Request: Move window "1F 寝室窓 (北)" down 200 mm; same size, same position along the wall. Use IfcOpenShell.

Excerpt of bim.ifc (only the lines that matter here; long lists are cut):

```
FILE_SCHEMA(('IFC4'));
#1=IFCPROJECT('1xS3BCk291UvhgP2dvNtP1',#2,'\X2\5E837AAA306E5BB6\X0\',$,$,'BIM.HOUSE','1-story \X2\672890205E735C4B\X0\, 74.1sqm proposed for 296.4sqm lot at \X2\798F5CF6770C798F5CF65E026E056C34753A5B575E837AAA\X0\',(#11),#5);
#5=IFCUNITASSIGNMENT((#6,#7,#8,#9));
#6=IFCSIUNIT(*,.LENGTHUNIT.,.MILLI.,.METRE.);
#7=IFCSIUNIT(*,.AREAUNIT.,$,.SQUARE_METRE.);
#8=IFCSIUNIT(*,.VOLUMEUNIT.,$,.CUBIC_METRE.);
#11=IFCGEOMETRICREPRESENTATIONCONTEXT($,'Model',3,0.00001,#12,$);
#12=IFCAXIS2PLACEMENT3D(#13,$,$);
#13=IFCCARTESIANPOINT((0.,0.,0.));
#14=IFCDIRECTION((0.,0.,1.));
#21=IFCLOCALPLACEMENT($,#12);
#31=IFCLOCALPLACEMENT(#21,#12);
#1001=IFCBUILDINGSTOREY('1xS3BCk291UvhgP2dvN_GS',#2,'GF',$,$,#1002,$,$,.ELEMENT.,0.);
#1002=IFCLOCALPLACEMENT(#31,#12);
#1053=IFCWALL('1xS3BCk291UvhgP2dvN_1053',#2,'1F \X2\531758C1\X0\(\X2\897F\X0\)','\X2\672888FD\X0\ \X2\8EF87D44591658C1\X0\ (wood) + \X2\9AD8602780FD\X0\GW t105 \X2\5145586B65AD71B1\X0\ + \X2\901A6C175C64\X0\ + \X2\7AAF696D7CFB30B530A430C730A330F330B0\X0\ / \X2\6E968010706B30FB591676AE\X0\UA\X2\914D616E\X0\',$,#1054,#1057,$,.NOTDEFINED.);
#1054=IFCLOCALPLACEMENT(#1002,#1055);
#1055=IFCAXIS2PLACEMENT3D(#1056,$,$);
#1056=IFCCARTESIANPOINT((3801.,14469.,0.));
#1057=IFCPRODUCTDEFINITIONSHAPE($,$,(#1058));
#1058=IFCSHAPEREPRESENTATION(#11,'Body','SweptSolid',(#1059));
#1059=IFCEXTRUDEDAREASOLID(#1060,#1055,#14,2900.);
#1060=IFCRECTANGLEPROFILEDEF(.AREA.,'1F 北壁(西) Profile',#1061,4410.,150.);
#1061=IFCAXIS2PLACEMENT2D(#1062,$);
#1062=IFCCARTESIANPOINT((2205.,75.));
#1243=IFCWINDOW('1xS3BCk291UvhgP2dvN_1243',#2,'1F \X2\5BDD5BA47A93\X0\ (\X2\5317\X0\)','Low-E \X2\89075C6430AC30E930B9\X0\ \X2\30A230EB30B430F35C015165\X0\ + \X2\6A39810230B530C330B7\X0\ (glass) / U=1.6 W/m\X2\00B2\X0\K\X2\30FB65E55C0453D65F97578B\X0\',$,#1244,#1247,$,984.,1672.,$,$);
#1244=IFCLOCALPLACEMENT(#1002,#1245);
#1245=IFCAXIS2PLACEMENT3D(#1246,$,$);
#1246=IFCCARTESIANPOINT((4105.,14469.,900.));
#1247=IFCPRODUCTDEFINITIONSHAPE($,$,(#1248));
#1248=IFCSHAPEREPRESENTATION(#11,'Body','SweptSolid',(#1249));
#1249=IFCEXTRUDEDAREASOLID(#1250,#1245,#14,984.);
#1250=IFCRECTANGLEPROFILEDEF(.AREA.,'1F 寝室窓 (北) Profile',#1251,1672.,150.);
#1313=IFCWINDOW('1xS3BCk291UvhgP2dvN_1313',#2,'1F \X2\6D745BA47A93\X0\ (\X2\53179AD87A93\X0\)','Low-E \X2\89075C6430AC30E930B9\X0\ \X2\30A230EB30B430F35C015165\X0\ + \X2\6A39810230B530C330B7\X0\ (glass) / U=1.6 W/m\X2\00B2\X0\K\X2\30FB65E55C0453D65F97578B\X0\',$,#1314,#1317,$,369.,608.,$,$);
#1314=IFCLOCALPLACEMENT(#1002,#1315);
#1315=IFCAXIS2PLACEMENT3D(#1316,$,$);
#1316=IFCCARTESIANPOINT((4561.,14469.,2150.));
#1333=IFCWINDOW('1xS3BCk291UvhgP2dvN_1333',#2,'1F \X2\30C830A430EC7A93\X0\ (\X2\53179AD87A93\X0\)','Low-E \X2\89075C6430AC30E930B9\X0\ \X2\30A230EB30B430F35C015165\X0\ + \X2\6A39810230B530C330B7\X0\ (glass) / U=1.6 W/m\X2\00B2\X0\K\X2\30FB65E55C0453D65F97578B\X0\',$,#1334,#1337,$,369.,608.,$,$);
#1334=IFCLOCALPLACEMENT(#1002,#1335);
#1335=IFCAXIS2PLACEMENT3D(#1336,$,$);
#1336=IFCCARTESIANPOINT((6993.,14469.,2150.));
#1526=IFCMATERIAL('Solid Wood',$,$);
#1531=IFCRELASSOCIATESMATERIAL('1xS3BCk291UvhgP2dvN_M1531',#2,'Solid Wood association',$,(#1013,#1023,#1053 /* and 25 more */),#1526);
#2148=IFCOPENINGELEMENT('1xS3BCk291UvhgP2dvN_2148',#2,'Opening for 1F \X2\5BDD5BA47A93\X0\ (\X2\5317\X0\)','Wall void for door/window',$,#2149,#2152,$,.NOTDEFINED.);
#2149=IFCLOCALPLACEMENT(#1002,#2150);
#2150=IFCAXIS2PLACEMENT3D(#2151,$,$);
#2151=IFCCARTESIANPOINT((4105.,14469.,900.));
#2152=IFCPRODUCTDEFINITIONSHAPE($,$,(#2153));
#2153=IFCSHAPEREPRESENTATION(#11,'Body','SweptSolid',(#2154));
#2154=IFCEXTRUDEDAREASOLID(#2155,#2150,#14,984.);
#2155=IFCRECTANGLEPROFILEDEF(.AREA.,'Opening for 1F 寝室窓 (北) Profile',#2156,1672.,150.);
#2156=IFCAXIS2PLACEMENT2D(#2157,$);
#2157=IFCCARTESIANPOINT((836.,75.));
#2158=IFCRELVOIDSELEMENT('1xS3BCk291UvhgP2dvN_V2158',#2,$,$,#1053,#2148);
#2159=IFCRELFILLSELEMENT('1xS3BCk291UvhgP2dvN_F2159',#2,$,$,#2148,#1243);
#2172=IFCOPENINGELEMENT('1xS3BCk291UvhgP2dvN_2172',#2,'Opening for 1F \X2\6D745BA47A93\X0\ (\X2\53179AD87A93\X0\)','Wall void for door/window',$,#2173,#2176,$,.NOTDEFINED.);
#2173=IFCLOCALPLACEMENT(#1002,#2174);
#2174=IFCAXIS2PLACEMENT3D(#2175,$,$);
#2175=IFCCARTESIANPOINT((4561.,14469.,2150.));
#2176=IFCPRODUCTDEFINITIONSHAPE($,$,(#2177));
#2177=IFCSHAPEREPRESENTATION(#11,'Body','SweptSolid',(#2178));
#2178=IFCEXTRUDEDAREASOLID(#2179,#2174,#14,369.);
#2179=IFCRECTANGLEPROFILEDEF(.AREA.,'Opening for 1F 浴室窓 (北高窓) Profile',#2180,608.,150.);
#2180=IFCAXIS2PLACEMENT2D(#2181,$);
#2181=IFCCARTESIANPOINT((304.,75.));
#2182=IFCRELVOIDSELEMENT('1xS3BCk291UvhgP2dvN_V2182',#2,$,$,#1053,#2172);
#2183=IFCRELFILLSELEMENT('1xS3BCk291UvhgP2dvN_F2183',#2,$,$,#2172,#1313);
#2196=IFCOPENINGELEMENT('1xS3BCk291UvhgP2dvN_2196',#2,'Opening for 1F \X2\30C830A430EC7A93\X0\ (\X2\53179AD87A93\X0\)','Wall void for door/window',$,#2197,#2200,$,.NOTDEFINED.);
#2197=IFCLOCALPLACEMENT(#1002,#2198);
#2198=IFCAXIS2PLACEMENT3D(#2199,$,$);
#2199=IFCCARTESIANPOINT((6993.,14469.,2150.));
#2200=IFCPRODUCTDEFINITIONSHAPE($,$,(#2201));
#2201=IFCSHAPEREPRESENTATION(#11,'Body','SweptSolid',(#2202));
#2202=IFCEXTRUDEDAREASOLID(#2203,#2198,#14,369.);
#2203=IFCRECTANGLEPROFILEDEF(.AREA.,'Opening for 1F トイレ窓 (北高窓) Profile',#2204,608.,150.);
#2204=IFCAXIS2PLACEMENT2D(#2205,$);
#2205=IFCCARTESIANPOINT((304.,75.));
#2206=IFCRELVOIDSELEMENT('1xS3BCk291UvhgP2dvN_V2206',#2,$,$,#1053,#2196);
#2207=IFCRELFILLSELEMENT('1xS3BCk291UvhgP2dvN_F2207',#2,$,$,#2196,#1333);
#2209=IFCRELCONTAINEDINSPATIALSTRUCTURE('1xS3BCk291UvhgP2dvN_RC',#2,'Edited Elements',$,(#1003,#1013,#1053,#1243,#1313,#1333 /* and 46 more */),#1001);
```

```python
import numpy as np
import ifcopenshell
import ifcopenshell.api.geometry
import ifcopenshell.util.placement
import ifcopenshell.util.unit

model = ifcopenshell.open("bim.ifc")
unit_scale = ifcopenshell.util.unit.calculate_unit_scale(model)

window = model.by_id(1243)
opening = window.FillsVoids[0].RelatingOpeningElement
dz = -200.0

shift = np.array([0.0, 0.0, dz])
# The window is not placed relative to its opening, so move both.
for product in (opening, window):
    matrix = ifcopenshell.util.placement.get_local_placement(product.ObjectPlacement)
    matrix[:3, 3] += shift
    ifcopenshell.api.geometry.edit_object_placement(model, product=product, matrix=matrix, is_si=False)

print(f"moved by {dz * unit_scale:+.3f} m")

model.write("bim_edited.ifc")
```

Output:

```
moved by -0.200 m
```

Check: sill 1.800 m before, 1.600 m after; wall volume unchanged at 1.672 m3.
